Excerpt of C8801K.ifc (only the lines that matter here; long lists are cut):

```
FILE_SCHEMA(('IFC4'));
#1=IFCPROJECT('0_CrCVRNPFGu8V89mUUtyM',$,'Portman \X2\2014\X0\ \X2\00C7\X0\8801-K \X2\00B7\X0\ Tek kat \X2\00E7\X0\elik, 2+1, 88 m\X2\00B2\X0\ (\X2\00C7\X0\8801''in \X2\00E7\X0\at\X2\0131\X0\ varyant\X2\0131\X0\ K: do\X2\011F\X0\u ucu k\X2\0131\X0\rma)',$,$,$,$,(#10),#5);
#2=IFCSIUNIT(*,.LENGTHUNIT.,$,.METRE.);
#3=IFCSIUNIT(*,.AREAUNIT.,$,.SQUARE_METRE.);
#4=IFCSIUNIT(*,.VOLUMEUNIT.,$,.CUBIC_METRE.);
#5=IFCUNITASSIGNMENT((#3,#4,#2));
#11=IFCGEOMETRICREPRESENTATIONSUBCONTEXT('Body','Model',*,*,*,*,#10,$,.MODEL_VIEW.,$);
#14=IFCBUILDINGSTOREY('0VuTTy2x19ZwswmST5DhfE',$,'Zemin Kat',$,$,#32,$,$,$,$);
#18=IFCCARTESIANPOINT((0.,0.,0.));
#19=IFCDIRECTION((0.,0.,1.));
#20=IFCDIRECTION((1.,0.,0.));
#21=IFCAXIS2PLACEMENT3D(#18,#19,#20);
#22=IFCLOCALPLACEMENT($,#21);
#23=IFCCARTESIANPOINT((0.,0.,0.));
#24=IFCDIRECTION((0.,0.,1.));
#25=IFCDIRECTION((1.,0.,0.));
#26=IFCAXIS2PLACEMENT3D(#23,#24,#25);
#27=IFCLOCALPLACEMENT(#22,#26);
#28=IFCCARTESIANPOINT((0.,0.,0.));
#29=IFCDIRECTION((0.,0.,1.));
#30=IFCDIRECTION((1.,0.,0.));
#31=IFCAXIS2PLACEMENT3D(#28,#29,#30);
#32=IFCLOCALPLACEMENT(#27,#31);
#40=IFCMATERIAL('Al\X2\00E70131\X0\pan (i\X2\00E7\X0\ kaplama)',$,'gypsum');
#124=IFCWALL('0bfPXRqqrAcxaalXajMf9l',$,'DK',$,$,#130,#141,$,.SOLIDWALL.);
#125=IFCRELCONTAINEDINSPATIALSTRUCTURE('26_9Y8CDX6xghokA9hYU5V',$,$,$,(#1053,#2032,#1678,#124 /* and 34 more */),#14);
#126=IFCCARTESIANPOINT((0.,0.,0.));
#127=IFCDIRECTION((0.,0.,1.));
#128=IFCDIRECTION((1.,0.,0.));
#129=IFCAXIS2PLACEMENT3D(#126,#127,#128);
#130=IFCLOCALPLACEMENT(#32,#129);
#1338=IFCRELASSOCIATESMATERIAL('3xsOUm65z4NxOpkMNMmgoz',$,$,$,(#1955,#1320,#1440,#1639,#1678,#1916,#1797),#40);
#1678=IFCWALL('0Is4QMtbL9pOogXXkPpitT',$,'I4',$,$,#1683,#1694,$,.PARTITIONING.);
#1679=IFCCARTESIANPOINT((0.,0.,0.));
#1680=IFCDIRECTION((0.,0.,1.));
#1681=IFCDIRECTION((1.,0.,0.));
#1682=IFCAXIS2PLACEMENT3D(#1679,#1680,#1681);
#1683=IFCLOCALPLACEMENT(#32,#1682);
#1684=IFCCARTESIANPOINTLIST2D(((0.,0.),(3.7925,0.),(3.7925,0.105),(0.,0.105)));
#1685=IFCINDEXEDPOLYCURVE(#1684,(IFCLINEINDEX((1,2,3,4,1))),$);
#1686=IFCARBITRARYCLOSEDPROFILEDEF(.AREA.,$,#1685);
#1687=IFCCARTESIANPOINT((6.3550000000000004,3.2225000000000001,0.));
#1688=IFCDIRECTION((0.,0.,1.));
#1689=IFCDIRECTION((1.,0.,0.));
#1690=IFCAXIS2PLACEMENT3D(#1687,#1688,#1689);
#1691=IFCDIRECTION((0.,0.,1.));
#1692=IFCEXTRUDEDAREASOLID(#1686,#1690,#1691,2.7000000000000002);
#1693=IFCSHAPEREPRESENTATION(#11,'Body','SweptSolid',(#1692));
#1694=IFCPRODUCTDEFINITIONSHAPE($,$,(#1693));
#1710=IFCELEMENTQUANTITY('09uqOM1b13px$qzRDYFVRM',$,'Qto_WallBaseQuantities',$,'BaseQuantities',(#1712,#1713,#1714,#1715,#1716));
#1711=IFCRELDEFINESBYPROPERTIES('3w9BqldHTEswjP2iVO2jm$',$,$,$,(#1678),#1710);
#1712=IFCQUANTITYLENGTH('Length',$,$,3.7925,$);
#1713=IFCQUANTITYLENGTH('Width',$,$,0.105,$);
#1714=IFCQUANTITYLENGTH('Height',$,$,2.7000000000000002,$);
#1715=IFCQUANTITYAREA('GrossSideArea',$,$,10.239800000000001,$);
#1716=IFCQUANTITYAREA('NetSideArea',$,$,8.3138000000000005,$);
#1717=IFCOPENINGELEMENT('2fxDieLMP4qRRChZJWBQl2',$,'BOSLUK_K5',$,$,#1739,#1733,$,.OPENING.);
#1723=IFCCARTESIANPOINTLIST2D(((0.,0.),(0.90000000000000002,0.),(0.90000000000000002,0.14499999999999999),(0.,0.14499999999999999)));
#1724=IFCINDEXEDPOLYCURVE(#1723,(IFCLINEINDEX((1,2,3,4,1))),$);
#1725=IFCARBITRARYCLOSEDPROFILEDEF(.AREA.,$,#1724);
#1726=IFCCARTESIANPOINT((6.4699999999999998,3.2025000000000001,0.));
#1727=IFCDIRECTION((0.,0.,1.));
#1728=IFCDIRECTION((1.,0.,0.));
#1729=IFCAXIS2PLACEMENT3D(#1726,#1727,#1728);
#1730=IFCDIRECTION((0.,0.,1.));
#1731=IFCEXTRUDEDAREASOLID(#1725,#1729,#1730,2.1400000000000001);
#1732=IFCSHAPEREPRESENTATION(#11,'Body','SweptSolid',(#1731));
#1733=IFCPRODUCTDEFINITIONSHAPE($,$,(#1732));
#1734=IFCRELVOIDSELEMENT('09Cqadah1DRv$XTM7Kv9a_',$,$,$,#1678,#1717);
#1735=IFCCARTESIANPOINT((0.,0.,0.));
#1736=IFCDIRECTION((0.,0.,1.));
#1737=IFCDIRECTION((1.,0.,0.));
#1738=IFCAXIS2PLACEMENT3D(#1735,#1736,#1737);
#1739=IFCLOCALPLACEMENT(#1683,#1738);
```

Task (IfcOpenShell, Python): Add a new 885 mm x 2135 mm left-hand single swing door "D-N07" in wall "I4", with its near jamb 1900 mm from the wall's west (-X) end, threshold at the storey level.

```python
import numpy as np
import ifcopenshell
import ifcopenshell.api.feature
import ifcopenshell.api.geometry
import ifcopenshell.api.pset
import ifcopenshell.api.root
import ifcopenshell.api.spatial
import ifcopenshell.geom
import ifcopenshell.util.element
import ifcopenshell.util.placement
import ifcopenshell.util.representation
import ifcopenshell.util.shape
import ifcopenshell.util.unit

model = ifcopenshell.open("C8801K.ifc")
unit_scale = ifcopenshell.util.unit.calculate_unit_scale(model)
area_scale = ifcopenshell.util.unit.calculate_unit_scale(model, "AREAUNIT")
settings = ifcopenshell.geom.settings()


def volume(element):
    """Net volume in cubic metres, openings subtracted."""
    shape = ifcopenshell.geom.create_shape(settings, element)
    return ifcopenshell.util.shape.get_volume(shape.geometry)


wall = model.by_guid("0Is4QMtbL9pOogXXkPpitT")
storey = ifcopenshell.util.element.get_container(wall, ifc_class="IfcBuildingStorey")
context = ifcopenshell.util.representation.get_context(model, "Model", "Body", "MODEL_VIEW")
before = volume(wall)

width, height, from_end, sill = 0.885, 2.135, 1.9, 0.0  # metres

# The wall runs along its own X axis, and the end named is its -X end.
wall_shape = ifcopenshell.geom.create_shape(settings, wall)
x, y, z = ifcopenshell.util.shape.get_vertices(wall_shape.geometry).T
start = x.min() + from_end
face, thickness = float(y.min()), float(y.max() - y.min())
wall_matrix = ifcopenshell.util.placement.get_local_placement(wall.ObjectPlacement)
level = ifcopenshell.util.placement.get_local_placement(storey.ObjectPlacement)[2, 3]


def in_wall(x, y):
    """Placement at x, y metres in the wall's axes, at sill height."""
    matrix = wall_matrix.copy()
    matrix[:, 3] = wall_matrix @ np.array([x / unit_scale, y / unit_scale, 0.0, 1.0])
    matrix[2, 3] = level + sill / unit_scale
    return matrix


# Opening: a box that overshoots both wall faces by 50 mm.
opening = ifcopenshell.api.root.create_entity(model, ifc_class="IfcOpeningElement", predefined_type="OPENING")
box = ifcopenshell.api.geometry.add_wall_representation(
    model, context=context, length=width, height=height, thickness=thickness + 0.1
)
ifcopenshell.api.geometry.assign_representation(model, product=opening, representation=box)
ifcopenshell.api.geometry.edit_object_placement(model, product=opening, matrix=in_wall(start, face - 0.05), is_si=False)
ifcopenshell.api.feature.add_feature(model, feature=opening, element=wall)

door = ifcopenshell.api.root.create_entity(model, ifc_class="IfcDoor", name="D-N07", predefined_type="DOOR")
door.OverallWidth, door.OverallHeight = width / unit_scale, height / unit_scale
door.OperationType = "SINGLE_SWING_LEFT"
body = ifcopenshell.api.geometry.add_door_representation(
    model,
    context=context,
    overall_width=door.OverallWidth,
    overall_height=door.OverallHeight,
    operation_type="SINGLE_SWING_LEFT",
    lining_properties={"LiningDepth": thickness / unit_scale, "ThresholdDepth": thickness / unit_scale},
)
ifcopenshell.api.geometry.assign_representation(model, product=door, representation=body)
ifcopenshell.api.spatial.assign_container(model, products=[door], relating_structure=storey)
ifcopenshell.api.feature.add_filling(model, opening=opening, element=door)

# The lining spans the wall, so the door starts at the wall face.
ifcopenshell.api.geometry.edit_object_placement(model, product=door, matrix=in_wall(start, face), is_si=False)

after = volume(wall)

# Update the wall's stored quantities.
qto = model.by_id(ifcopenshell.util.element.get_pset(wall, "Qto_WallBaseQuantities", should_inherit=False)["id"])
ifcopenshell.api.pset.edit_qto(model, qto=qto, properties={"NetSideArea": after / thickness / area_scale})

print(f"wall volume {before:.3f} -> {after:.3f} m3")

model.write("C8801K-out.ifc")
```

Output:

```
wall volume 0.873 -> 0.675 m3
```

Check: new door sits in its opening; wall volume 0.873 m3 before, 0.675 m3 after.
